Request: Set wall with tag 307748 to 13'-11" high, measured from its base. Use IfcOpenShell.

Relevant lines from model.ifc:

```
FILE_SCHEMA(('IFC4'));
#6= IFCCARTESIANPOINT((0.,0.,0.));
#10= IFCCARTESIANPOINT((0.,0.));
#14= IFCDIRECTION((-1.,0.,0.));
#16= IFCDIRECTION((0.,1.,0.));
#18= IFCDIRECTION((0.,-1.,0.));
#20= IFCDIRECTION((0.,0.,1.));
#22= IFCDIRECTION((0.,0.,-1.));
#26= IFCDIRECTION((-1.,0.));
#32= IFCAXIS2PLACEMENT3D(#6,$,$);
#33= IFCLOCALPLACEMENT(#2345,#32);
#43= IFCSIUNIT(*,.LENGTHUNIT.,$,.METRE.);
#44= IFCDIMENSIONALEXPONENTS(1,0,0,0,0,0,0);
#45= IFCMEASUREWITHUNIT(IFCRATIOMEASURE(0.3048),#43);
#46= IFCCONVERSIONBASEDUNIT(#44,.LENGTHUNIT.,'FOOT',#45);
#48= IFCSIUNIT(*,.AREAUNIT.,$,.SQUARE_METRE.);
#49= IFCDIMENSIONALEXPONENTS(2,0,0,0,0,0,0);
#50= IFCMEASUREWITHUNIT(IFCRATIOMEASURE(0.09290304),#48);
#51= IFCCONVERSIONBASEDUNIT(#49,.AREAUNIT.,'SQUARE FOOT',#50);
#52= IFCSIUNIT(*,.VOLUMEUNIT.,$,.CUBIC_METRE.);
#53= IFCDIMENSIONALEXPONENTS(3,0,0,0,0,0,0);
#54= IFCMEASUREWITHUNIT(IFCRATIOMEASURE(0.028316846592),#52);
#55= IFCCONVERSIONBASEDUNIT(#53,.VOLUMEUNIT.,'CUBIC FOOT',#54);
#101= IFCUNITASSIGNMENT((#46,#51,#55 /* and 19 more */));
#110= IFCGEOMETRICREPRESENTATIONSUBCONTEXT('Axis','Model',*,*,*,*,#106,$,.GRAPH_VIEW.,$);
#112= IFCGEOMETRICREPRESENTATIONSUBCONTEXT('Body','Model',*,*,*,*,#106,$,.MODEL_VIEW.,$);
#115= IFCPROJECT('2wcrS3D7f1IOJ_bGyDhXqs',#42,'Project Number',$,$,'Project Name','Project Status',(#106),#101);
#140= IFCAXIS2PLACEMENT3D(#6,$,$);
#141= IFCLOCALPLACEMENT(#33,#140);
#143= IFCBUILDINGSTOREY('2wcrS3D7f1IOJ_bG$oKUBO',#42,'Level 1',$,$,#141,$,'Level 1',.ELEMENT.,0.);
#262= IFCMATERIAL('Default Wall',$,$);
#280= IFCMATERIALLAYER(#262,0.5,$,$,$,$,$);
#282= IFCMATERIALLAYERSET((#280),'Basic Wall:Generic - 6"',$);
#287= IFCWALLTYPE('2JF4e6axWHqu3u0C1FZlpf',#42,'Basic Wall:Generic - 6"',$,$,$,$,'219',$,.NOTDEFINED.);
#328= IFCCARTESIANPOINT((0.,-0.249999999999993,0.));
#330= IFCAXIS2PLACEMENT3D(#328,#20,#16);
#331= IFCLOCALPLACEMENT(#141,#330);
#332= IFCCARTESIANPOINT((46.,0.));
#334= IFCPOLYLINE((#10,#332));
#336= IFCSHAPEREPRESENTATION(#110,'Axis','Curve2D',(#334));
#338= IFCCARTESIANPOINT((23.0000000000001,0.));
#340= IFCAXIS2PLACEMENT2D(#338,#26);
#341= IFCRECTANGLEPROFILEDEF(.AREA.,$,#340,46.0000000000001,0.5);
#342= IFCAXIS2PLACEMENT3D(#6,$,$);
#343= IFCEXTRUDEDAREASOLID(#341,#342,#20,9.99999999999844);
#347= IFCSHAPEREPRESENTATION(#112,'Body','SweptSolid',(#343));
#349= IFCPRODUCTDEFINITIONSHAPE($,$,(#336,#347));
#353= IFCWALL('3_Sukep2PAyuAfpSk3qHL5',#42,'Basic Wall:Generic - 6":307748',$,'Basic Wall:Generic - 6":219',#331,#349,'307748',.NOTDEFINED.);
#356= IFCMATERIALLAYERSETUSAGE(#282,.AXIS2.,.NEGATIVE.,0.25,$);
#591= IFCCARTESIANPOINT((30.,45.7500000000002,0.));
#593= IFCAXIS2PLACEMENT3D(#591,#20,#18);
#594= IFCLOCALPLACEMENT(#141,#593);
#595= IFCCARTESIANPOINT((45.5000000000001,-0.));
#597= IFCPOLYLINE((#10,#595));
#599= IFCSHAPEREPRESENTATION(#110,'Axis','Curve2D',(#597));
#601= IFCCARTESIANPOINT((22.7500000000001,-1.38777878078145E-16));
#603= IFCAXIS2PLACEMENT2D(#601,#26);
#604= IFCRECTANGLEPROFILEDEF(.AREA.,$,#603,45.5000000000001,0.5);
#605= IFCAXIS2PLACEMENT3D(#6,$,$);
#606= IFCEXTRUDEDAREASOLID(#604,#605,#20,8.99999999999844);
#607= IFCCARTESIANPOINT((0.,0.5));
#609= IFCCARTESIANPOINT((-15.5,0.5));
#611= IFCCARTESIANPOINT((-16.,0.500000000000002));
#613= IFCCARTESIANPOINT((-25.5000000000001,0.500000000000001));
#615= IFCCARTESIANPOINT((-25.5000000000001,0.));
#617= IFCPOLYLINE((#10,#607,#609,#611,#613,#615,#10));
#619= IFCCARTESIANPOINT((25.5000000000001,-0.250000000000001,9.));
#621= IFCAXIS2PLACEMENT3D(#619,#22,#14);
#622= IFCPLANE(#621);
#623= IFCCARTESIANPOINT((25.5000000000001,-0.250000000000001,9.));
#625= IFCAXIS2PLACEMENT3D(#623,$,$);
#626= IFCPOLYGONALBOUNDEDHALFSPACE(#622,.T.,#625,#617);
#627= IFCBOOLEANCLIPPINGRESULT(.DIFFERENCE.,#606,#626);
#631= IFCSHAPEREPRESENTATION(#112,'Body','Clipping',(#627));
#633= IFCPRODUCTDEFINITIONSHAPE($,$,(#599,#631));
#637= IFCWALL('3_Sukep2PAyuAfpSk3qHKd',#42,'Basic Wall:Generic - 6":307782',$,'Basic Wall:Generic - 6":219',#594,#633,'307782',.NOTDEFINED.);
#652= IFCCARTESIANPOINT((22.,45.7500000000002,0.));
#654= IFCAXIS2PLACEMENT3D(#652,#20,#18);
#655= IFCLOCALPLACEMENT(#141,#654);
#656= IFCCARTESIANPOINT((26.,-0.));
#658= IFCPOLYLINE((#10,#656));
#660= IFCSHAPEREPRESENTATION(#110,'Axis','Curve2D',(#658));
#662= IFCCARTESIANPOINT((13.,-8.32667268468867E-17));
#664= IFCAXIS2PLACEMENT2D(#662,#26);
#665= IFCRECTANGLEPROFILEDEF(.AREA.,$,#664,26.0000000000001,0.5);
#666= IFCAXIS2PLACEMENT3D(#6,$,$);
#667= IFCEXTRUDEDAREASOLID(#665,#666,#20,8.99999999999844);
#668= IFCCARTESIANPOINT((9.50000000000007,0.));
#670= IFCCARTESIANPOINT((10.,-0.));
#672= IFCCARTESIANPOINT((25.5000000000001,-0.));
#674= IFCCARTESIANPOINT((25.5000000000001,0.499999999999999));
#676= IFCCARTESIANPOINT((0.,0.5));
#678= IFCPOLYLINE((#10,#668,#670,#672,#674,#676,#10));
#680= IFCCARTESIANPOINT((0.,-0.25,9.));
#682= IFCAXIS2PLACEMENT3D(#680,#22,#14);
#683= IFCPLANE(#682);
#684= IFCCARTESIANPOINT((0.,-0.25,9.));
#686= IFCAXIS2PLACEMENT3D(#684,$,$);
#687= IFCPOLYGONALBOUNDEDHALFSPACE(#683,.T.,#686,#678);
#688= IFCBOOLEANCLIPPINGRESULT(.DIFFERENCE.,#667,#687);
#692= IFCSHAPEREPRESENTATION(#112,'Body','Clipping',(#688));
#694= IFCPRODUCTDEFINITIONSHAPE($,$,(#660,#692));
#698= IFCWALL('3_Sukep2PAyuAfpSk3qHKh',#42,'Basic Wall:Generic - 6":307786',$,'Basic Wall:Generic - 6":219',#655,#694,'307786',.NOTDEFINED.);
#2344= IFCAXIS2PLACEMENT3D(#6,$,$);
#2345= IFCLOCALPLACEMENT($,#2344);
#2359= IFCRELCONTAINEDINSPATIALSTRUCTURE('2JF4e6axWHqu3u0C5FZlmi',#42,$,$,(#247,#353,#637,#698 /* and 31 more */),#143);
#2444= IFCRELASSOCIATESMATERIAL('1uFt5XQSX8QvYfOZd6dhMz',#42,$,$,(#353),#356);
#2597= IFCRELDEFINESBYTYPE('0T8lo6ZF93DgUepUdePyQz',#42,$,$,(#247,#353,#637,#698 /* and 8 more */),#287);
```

```python
import ifcopenshell
import ifcopenshell.geom
import ifcopenshell.util.representation
import ifcopenshell.util.shape
import ifcopenshell.util.unit

model = ifcopenshell.open("model.ifc")
unit_scale = ifcopenshell.util.unit.calculate_unit_scale(model)
settings = ifcopenshell.geom.settings()


def volume(element):
    """Net volume in cubic metres, openings subtracted."""
    shape = ifcopenshell.geom.create_shape(settings, element)
    return ifcopenshell.util.shape.get_volume(shape.geometry)


wall = model.by_guid("3_Sukep2PAyuAfpSk3qHL5")
before = volume(wall)

body = ifcopenshell.util.representation.get_representation(wall, "Model", "Body")
solid = body.Items[0]
old_height = solid.Depth
solid.Depth = 167 * 0.0254 / unit_scale
after = volume(wall)

print(f"height {old_height:g} -> {solid.Depth:g}, volume {before:.3f} -> {after:.3f} m3")

model.write("model_updated.ifc")
```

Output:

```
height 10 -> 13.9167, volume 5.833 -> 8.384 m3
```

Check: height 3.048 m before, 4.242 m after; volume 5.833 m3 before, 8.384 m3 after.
